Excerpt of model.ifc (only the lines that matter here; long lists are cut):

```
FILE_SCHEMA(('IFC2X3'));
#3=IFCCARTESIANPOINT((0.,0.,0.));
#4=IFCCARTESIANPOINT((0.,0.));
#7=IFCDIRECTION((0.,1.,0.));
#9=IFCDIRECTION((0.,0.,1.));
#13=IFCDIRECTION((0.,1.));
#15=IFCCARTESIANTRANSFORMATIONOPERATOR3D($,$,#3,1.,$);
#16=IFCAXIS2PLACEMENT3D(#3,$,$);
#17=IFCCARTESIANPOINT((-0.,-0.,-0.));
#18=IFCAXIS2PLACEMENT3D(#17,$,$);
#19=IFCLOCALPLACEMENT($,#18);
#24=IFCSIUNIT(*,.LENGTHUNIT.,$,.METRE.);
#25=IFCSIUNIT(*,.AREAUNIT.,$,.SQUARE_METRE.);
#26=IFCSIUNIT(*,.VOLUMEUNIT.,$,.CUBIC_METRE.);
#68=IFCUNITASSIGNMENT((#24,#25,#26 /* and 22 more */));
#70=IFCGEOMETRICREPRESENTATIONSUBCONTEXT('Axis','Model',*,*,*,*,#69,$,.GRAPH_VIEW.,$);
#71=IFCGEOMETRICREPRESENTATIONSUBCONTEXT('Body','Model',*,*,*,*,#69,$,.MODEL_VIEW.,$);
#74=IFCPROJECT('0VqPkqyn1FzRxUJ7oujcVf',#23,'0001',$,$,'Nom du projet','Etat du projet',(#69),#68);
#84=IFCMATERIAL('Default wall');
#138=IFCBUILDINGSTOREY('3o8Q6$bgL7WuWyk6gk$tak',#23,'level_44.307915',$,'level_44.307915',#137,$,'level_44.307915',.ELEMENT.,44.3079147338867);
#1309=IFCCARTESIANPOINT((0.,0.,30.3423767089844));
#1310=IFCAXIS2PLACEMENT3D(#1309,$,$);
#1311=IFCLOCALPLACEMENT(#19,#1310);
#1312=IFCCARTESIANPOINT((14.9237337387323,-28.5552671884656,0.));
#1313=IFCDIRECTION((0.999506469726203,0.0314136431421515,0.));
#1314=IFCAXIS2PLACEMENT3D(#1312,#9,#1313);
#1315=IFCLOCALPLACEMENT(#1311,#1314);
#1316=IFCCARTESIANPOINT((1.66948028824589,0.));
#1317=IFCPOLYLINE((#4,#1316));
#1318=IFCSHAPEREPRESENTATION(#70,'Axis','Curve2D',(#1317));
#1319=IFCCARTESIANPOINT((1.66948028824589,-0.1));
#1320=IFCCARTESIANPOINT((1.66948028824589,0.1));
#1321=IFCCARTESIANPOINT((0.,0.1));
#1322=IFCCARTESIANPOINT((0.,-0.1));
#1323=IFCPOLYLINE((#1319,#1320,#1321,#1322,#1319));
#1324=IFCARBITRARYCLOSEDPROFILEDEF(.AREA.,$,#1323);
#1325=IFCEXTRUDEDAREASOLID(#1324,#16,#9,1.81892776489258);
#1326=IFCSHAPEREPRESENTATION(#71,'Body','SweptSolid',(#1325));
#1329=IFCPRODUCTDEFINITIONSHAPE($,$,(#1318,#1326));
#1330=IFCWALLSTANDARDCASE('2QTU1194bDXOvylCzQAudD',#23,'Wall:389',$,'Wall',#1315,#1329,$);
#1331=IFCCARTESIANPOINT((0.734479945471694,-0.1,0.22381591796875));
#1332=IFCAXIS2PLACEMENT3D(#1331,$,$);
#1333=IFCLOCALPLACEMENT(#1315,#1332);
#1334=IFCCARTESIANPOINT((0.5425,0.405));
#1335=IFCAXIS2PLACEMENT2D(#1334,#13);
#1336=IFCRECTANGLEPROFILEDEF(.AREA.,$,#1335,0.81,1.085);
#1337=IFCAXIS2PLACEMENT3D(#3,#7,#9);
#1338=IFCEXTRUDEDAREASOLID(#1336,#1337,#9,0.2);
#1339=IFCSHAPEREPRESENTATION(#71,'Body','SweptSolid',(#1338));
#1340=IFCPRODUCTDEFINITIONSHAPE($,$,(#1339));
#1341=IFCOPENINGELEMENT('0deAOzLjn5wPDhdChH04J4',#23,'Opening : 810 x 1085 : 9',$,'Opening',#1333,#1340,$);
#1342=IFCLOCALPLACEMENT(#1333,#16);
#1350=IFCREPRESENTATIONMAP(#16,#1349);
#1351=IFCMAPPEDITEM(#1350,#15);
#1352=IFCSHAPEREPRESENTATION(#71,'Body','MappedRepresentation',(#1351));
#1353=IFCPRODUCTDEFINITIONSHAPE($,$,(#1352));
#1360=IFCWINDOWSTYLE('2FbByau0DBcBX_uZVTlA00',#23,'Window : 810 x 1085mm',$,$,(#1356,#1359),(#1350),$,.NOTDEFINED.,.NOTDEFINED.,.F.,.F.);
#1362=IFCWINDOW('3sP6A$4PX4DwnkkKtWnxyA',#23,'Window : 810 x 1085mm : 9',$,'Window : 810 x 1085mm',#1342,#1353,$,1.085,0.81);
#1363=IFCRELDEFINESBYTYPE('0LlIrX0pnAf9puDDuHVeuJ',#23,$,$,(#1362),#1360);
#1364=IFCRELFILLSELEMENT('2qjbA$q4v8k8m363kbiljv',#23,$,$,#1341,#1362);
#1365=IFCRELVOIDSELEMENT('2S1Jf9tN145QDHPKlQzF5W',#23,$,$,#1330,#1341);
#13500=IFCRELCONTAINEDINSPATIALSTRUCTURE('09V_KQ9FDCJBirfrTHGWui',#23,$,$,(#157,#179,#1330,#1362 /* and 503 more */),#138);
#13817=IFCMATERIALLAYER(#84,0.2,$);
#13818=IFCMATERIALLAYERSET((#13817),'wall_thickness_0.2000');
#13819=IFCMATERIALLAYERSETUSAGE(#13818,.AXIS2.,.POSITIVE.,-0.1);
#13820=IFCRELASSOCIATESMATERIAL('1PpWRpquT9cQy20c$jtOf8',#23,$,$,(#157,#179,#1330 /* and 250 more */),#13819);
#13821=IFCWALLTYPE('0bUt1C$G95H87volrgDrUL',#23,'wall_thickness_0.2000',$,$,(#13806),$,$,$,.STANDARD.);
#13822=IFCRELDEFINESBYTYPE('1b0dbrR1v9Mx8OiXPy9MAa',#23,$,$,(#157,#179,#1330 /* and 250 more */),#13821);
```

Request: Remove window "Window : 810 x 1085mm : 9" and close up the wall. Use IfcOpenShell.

```python
import ifcopenshell
import ifcopenshell.api.feature
import ifcopenshell.api.root
import ifcopenshell.geom
import ifcopenshell.util.shape

model = ifcopenshell.open("model.ifc")
settings = ifcopenshell.geom.settings()


def volume(element):
    """Net volume in cubic metres, openings subtracted."""
    shape = ifcopenshell.geom.create_shape(settings, element)
    return ifcopenshell.util.shape.get_volume(shape.geometry)


window = model.by_guid("3sP6A$4PX4DwnkkKtWnxyA")
opening = window.FillsVoids[0].RelatingOpeningElement
wall = opening.VoidsElements[0].RelatingBuildingElement
before = volume(wall)

ifcopenshell.api.root.remove_product(model, product=window)
ifcopenshell.api.feature.remove_feature(model, feature=opening)

after = volume(wall)

print(f"wall volume {before:.3f} -> {after:.3f} m3")

model.write("model_updated.ifc")
```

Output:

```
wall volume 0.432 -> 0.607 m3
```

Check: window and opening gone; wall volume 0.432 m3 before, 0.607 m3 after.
